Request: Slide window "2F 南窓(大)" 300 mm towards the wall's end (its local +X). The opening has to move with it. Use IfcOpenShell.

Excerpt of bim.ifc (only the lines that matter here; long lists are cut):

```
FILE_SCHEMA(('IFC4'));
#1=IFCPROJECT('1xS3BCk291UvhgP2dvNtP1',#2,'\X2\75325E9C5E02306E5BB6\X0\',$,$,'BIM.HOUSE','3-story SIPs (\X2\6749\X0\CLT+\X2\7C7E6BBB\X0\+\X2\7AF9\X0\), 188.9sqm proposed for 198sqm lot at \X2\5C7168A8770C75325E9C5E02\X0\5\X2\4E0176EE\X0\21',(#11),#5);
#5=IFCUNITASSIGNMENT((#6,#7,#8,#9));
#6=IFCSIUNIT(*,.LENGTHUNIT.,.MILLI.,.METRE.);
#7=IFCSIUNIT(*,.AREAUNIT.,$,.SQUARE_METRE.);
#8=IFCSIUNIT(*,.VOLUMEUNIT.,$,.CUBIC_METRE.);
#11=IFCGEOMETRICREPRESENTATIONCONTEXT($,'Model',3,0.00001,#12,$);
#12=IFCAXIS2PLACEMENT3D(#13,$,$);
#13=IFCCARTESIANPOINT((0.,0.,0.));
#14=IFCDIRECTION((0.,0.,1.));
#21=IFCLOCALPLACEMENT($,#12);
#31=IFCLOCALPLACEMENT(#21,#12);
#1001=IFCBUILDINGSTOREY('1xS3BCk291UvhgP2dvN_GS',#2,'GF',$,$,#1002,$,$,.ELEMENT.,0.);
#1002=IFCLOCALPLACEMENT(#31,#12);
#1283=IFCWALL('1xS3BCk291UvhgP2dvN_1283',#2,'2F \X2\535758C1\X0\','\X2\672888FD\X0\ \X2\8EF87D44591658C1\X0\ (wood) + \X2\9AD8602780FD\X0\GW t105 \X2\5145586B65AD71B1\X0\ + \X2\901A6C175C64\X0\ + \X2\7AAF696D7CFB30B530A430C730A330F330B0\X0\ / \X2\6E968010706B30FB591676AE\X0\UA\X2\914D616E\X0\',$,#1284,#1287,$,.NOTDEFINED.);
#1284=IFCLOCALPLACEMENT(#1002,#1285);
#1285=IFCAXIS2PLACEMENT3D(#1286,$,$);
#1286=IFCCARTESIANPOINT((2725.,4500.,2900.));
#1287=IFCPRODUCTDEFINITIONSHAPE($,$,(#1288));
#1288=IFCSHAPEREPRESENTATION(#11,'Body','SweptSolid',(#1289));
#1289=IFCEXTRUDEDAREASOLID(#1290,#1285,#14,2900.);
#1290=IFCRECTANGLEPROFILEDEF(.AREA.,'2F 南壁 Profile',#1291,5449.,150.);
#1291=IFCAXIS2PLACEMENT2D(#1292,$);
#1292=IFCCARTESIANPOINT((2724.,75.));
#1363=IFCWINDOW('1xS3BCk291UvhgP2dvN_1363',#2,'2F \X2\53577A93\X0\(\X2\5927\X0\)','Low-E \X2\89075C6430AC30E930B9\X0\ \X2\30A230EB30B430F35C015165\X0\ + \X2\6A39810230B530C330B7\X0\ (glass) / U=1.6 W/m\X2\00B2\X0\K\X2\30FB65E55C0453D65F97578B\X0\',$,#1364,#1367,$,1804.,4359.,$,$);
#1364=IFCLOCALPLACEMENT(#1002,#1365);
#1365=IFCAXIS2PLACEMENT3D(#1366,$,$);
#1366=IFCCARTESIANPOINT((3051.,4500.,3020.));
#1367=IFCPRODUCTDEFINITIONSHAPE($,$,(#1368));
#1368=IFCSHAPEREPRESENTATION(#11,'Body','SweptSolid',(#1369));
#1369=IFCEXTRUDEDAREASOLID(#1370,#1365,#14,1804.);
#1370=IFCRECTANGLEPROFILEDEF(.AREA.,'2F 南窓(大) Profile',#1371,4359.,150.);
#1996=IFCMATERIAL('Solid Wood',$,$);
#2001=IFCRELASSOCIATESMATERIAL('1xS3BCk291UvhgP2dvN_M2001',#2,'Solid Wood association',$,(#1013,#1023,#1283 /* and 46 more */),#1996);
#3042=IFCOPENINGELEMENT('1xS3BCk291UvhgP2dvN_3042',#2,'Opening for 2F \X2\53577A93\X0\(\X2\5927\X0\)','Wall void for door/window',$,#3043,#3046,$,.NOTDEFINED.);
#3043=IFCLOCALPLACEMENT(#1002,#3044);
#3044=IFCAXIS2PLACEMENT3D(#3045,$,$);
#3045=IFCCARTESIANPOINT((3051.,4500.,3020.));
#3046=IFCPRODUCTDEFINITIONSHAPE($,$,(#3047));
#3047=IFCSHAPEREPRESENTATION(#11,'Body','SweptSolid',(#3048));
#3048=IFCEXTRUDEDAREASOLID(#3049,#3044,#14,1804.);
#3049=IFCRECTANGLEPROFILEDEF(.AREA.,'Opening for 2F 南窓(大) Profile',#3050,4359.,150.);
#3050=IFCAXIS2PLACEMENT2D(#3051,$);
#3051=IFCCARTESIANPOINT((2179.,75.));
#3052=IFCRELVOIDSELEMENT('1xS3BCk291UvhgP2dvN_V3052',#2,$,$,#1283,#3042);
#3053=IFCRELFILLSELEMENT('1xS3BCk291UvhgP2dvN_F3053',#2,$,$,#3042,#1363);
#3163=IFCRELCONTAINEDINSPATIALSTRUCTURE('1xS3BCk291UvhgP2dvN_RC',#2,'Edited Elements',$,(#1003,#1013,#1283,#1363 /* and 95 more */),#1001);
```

```python
import ifcopenshell
import ifcopenshell.api.geometry
import ifcopenshell.util.placement

model = ifcopenshell.open("bim.ifc")

window = model.by_guid("1xS3BCk291UvhgP2dvN_1363")
opening = window.FillsVoids[0].RelatingOpeningElement
wall = opening.VoidsElements[0].RelatingBuildingElement

wall_matrix = ifcopenshell.util.placement.get_local_placement(wall.ObjectPlacement)
shift = wall_matrix[:3, 0] * 300.0
before = ifcopenshell.util.placement.get_local_placement(window.ObjectPlacement)[:3, 3].copy()

# The window is not placed relative to its opening, so move both.
for product in (opening, window):
    matrix = ifcopenshell.util.placement.get_local_placement(product.ObjectPlacement)
    matrix[:3, 3] += shift
    ifcopenshell.api.geometry.edit_object_placement(model, product=product, matrix=matrix, is_si=False)

after = ifcopenshell.util.placement.get_local_placement(window.ObjectPlacement)[:3, 3]
print("window moved by", (after - before).round(3) + 0.0)

model.write("bim_v2.ifc")
```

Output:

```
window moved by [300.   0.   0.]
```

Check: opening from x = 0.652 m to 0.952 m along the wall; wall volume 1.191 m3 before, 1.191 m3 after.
